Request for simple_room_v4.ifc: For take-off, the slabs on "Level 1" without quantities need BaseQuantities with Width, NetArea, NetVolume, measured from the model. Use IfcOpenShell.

First a look at what the model holds.

```python
import ifcopenshell
import ifcopenshell.util.element
import ifcopenshell.util.unit

model = ifcopenshell.open("simple_room_v4.ifc")
print(model.schema)
for unit_type in ("LENGTHUNIT", "AREAUNIT", "VOLUMEUNIT"):
    print(unit_type, ifcopenshell.util.unit.calculate_unit_scale(model, unit_type))
storey = next(s for s in model.by_type("IfcBuildingStorey") if s.Name == "Level 1")
slabs = [e for e in ifcopenshell.util.element.get_decomposition(storey) if e.is_a("IfcSlab")]
for e in sorted(slabs, key=lambda e: e.id()):
    print(e.id(), e.is_a(), e.Name, list(ifcopenshell.util.element.get_psets(e, qtos_only=True)), sep=" | ")
```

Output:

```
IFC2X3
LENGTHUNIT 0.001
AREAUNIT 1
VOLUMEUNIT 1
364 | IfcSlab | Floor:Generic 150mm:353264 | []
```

```python
import ifcopenshell
import ifcopenshell.api.pset
import ifcopenshell.geom
import ifcopenshell.util.element
import ifcopenshell.util.shape
import ifcopenshell.util.unit

model = ifcopenshell.open("simple_room_v4.ifc")
unit_scale = ifcopenshell.util.unit.calculate_unit_scale(model)
area_scale = ifcopenshell.util.unit.calculate_unit_scale(model, "AREAUNIT")
volume_scale = ifcopenshell.util.unit.calculate_unit_scale(model, "VOLUMEUNIT")
settings = ifcopenshell.geom.settings()

storey = next(s for s in model.by_type("IfcBuildingStorey") if s.Name == "Level 1")
slabs = [e for e in ifcopenshell.util.element.get_decomposition(storey) if e.is_a("IfcSlab")]

for e in sorted(slabs, key=lambda e: e.id()):
    if ifcopenshell.util.element.get_psets(e, qtos_only=True, should_inherit=False):
        continue
    # Geometry comes back in metres, in the element's own axes.
    shape = ifcopenshell.geom.create_shape(settings, e)
    values = {
        "Width": ifcopenshell.util.shape.get_z(shape.geometry) / unit_scale,
        "NetArea": ifcopenshell.util.shape.get_footprint_area(shape.geometry) / area_scale,
        "NetVolume": ifcopenshell.util.shape.get_volume(shape.geometry) / volume_scale,
    }
    qto = ifcopenshell.api.pset.add_qto(model, product=e, name="BaseQuantities")
    ifcopenshell.api.pset.edit_qto(model, qto=qto, properties=values)
    print(e.id(), {k: round(v, 3) for k, v in values.items()})

model.write("simple_room_v4_updated.ifc")
```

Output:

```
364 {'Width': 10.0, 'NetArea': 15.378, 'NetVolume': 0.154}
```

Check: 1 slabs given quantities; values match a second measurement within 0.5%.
